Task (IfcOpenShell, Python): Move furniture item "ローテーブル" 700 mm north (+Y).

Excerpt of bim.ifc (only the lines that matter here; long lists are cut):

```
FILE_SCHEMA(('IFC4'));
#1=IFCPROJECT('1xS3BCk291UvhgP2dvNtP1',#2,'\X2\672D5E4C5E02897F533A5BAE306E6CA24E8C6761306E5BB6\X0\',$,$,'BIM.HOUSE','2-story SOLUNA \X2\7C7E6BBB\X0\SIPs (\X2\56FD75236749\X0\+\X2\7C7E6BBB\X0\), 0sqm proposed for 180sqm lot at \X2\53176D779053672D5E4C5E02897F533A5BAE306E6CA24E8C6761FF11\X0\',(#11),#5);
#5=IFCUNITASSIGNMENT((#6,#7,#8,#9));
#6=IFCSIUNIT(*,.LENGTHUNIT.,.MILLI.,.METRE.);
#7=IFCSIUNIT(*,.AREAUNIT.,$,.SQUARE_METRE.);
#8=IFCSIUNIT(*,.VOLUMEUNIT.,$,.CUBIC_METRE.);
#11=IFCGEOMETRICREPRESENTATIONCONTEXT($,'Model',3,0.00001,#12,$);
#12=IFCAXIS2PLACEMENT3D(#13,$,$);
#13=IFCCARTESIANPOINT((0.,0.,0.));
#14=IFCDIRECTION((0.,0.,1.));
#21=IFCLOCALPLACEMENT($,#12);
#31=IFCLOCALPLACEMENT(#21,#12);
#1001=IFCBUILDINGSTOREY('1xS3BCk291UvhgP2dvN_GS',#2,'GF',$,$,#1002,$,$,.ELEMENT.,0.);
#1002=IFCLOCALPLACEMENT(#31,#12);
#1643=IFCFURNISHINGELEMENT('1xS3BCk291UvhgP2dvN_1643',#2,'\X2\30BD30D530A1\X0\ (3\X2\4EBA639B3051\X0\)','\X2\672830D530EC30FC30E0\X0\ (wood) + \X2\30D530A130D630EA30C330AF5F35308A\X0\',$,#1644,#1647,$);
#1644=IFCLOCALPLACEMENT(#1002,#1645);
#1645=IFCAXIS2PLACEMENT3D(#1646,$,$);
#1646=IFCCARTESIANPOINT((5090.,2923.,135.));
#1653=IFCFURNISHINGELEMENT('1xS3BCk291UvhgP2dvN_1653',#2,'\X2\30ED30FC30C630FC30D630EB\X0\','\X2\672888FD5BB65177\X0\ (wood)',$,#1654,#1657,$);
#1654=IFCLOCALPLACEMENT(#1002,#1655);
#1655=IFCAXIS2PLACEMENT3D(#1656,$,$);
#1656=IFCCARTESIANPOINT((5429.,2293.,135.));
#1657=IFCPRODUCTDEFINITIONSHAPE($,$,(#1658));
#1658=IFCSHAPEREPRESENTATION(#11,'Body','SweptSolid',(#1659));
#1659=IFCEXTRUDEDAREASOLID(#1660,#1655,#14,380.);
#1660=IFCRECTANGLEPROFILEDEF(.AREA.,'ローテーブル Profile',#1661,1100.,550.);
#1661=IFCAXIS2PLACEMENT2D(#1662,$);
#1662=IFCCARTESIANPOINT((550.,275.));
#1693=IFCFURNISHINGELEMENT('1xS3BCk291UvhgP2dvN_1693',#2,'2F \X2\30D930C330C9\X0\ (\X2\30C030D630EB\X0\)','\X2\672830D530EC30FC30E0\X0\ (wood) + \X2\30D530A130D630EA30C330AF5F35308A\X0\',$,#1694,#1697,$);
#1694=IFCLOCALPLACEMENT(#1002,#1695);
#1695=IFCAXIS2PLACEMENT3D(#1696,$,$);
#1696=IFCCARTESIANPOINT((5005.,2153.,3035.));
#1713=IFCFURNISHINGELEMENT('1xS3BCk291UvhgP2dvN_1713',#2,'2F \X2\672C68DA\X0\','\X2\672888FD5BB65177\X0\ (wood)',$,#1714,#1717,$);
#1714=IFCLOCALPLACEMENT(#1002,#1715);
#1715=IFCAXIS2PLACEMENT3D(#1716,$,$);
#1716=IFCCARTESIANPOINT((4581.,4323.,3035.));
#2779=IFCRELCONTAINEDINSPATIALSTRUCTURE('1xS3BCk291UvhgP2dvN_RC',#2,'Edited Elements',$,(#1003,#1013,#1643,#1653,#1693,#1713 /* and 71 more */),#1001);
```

```python
import ifcopenshell
import ifcopenshell.api.geometry
import ifcopenshell.util.placement
import ifcopenshell.util.unit

model = ifcopenshell.open("bim.ifc")
unit_scale = ifcopenshell.util.unit.calculate_unit_scale(model)

item = model.by_guid("1xS3BCk291UvhgP2dvN_1653")
matrix = ifcopenshell.util.placement.get_local_placement(item.ObjectPlacement)
matrix[1, 3] += 0.7 / unit_scale
ifcopenshell.api.geometry.edit_object_placement(model, product=item, matrix=matrix, is_si=False)

print(ifcopenshell.util.placement.get_local_placement(item.ObjectPlacement).round(3) + 0.0)

model.write("bim_v2.ifc")
```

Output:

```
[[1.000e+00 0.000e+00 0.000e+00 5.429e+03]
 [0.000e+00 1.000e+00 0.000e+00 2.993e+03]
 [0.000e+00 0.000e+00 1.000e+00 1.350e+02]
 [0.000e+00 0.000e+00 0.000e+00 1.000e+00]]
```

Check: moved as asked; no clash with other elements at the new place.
